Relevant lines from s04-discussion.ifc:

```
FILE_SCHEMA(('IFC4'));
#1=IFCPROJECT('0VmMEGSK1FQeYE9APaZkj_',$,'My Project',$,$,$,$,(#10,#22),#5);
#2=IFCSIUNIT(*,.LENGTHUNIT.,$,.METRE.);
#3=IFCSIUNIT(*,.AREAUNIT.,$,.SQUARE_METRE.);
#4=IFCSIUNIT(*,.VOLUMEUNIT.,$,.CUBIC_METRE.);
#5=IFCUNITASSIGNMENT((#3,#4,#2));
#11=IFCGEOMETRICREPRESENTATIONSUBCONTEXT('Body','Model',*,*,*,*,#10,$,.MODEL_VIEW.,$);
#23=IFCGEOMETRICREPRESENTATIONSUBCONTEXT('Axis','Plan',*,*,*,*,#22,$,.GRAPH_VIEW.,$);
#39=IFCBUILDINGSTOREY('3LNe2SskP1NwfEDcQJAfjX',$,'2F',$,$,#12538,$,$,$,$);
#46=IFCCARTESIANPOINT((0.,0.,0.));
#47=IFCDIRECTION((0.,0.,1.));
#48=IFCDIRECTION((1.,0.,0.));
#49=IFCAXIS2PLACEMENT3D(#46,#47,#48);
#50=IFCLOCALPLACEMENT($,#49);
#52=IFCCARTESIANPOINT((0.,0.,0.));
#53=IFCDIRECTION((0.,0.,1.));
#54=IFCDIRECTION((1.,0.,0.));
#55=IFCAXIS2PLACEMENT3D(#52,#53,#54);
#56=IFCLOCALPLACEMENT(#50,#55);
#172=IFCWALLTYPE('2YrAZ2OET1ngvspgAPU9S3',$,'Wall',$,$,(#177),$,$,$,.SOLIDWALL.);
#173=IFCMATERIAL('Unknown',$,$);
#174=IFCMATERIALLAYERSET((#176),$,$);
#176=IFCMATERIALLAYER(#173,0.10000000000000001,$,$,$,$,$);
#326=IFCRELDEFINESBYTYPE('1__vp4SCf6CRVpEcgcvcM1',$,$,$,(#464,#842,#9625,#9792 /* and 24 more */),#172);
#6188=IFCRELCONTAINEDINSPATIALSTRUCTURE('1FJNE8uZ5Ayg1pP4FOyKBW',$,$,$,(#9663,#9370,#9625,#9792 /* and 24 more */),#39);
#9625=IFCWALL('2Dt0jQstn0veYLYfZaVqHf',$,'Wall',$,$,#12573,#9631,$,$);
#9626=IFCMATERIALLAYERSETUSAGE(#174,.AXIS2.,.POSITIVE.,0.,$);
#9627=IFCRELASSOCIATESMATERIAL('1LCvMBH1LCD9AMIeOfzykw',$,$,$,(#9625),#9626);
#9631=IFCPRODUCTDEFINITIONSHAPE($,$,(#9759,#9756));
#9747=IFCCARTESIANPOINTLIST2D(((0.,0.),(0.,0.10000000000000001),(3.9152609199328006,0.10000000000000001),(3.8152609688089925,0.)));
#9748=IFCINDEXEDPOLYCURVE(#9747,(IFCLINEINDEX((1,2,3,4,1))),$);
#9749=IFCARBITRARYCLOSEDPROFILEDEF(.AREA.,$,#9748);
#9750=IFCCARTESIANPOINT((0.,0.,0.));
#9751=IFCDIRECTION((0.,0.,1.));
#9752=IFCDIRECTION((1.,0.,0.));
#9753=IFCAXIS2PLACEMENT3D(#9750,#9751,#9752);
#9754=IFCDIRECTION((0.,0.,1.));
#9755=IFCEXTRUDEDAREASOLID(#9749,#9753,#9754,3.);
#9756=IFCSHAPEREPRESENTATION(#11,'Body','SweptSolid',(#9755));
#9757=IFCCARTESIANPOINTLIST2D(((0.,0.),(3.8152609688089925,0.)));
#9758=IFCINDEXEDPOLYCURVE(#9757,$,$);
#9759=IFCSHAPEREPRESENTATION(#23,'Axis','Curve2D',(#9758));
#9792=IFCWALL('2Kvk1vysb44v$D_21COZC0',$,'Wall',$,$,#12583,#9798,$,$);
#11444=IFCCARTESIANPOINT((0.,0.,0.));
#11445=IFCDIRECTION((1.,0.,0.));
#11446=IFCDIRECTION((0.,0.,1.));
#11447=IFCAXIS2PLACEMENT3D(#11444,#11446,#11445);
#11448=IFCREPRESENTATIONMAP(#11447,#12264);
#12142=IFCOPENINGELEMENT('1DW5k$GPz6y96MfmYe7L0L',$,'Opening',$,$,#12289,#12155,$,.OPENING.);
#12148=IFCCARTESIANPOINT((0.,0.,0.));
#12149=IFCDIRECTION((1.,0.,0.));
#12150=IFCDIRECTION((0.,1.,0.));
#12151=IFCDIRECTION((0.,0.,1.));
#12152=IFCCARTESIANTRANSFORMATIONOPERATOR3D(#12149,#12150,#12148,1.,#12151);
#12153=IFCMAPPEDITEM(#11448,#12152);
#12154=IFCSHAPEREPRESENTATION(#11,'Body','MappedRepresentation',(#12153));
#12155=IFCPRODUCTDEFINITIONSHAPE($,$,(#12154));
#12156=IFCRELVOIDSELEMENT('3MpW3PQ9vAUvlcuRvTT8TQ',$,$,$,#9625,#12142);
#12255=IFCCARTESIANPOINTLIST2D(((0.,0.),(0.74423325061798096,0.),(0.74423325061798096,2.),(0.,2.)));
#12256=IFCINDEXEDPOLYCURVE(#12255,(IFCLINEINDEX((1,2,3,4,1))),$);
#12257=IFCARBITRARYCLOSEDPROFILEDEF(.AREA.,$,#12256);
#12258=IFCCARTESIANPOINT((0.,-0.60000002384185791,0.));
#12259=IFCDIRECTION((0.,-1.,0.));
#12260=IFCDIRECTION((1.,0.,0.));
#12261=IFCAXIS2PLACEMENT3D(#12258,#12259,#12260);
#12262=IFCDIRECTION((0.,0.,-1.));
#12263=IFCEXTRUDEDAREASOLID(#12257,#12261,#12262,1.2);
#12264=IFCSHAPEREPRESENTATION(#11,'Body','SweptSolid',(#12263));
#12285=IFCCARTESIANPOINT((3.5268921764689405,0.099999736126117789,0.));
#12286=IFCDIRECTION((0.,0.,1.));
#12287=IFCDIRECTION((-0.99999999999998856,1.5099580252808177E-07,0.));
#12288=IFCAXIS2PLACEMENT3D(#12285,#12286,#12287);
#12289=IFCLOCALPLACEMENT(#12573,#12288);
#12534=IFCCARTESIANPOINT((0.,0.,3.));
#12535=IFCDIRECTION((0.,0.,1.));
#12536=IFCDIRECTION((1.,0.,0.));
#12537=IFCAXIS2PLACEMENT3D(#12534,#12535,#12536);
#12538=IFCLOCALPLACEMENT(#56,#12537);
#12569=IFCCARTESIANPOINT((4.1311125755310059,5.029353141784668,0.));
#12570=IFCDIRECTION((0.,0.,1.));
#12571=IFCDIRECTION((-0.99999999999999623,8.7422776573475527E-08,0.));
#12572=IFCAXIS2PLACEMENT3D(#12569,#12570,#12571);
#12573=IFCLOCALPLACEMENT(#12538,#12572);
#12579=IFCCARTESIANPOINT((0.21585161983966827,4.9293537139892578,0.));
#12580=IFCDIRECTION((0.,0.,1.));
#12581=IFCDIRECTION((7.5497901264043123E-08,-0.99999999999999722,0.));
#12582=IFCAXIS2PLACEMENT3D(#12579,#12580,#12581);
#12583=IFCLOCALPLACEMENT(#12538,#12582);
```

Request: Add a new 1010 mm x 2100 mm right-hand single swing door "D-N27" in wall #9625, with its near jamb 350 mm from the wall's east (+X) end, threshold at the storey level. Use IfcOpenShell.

```python
import numpy as np
import ifcopenshell
import ifcopenshell.api.feature
import ifcopenshell.api.geometry
import ifcopenshell.api.root
import ifcopenshell.api.spatial
import ifcopenshell.geom
import ifcopenshell.util.element
import ifcopenshell.util.placement
import ifcopenshell.util.representation
import ifcopenshell.util.shape
import ifcopenshell.util.unit

model = ifcopenshell.open("s04-discussion.ifc")
unit_scale = ifcopenshell.util.unit.calculate_unit_scale(model)
settings = ifcopenshell.geom.settings()


def volume(element):
    """Net volume in cubic metres, openings subtracted."""
    shape = ifcopenshell.geom.create_shape(settings, element)
    return ifcopenshell.util.shape.get_volume(shape.geometry)


wall = model.by_guid("2Dt0jQstn0veYLYfZaVqHf")
storey = ifcopenshell.util.element.get_container(wall, ifc_class="IfcBuildingStorey")
context = ifcopenshell.util.representation.get_context(model, "Model", "Body", "MODEL_VIEW")
before = volume(wall)

width, height, from_end, sill = 1.01, 2.1, 0.35, 0.0  # metres

# The wall runs along its own X axis, and the end named is its -X end.
wall_shape = ifcopenshell.geom.create_shape(settings, wall)
x, y, z = ifcopenshell.util.shape.get_vertices(wall_shape.geometry).T
start = x.min() + from_end
face, thickness = float(y.min()), float(y.max() - y.min())
wall_matrix = ifcopenshell.util.placement.get_local_placement(wall.ObjectPlacement)
level = ifcopenshell.util.placement.get_local_placement(storey.ObjectPlacement)[2, 3]


def in_wall(x, y):
    """Placement at x, y metres in the wall's axes, at sill height."""
    matrix = wall_matrix.copy()
    matrix[:, 3] = wall_matrix @ np.array([x / unit_scale, y / unit_scale, 0.0, 1.0])
    matrix[2, 3] = level + sill / unit_scale
    return matrix


# Opening: a box that overshoots both wall faces by 50 mm.
opening = ifcopenshell.api.root.create_entity(model, ifc_class="IfcOpeningElement", predefined_type="OPENING")
box = ifcopenshell.api.geometry.add_wall_representation(
    model, context=context, length=width, height=height, thickness=thickness + 0.1
)
ifcopenshell.api.geometry.assign_representation(model, product=opening, representation=box)
ifcopenshell.api.geometry.edit_object_placement(model, product=opening, matrix=in_wall(start, face - 0.05), is_si=False)
ifcopenshell.api.feature.add_feature(model, feature=opening, element=wall)

door = ifcopenshell.api.root.create_entity(model, ifc_class="IfcDoor", name="D-N27", predefined_type="DOOR")
door.OverallWidth, door.OverallHeight = width / unit_scale, height / unit_scale
door.OperationType = "SINGLE_SWING_RIGHT"
body = ifcopenshell.api.geometry.add_door_representation(
    model,
    context=context,
    overall_width=door.OverallWidth,
    overall_height=door.OverallHeight,
    operation_type="SINGLE_SWING_RIGHT",
    lining_properties={"LiningDepth": thickness / unit_scale, "ThresholdDepth": thickness / unit_scale},
)
ifcopenshell.api.geometry.assign_representation(model, product=door, representation=body)
ifcopenshell.api.spatial.assign_container(model, products=[door], relating_structure=storey)
ifcopenshell.api.feature.add_filling(model, opening=opening, element=door)

# The lining spans the wall, so the door starts at the wall face.
ifcopenshell.api.geometry.edit_object_placement(model, product=door, matrix=in_wall(start, face), is_si=False)

after = volume(wall)

print(f"wall volume {before:.3f} -> {after:.3f} m3")

model.write("s04-discussion-out.ifc")
```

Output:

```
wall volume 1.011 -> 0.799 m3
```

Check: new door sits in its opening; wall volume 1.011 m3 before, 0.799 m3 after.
